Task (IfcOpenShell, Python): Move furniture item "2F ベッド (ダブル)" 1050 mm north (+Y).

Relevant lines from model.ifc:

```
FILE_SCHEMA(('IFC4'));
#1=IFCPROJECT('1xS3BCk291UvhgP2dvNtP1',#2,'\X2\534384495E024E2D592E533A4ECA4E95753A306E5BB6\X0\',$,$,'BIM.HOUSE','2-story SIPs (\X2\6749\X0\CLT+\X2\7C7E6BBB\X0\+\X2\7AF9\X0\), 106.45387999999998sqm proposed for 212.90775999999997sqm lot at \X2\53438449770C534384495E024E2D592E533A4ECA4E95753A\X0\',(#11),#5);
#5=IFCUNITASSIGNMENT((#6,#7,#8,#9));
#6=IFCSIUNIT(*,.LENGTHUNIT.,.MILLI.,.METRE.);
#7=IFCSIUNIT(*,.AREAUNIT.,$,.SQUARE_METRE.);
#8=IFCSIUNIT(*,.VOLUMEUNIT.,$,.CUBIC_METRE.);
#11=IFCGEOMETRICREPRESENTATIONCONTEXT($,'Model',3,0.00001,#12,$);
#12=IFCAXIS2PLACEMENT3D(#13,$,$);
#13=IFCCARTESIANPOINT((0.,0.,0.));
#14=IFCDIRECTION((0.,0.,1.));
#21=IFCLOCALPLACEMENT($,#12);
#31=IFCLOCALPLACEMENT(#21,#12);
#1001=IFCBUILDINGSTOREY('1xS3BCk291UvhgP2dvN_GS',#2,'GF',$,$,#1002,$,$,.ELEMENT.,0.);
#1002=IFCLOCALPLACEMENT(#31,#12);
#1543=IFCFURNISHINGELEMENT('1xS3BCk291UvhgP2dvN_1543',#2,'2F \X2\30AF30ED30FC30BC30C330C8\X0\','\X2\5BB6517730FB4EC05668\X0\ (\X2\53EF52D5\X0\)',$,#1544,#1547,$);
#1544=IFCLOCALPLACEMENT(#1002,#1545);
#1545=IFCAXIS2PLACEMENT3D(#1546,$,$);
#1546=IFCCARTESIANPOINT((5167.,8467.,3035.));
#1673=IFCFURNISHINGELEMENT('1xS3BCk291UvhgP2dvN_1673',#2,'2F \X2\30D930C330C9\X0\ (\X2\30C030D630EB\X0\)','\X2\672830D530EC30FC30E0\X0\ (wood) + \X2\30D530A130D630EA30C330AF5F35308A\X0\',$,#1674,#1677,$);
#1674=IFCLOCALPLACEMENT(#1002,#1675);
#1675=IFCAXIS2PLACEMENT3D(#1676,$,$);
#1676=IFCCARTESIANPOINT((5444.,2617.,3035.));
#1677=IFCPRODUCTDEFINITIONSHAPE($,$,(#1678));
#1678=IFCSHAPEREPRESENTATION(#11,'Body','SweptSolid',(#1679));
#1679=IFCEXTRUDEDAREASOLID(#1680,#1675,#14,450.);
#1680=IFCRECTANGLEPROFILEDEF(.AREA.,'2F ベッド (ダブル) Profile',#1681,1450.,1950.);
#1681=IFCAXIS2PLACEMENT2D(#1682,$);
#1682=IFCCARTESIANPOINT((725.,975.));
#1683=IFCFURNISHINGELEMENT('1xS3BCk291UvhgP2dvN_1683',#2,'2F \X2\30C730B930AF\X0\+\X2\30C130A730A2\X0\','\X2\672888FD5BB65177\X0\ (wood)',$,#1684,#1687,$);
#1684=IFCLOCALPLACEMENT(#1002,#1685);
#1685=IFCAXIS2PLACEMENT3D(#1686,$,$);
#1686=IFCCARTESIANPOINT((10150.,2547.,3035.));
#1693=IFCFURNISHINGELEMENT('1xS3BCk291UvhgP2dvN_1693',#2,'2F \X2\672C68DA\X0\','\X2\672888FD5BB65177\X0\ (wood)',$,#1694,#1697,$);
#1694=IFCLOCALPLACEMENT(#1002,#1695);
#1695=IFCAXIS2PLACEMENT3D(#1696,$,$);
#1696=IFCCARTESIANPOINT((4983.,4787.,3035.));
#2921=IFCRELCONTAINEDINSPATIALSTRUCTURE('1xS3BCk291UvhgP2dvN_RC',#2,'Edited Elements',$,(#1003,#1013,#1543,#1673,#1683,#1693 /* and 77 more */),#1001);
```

```python
import ifcopenshell
import ifcopenshell.api.geometry
import ifcopenshell.util.placement
import ifcopenshell.util.unit

model = ifcopenshell.open("model.ifc")
unit_scale = ifcopenshell.util.unit.calculate_unit_scale(model)

item = model.by_guid("1xS3BCk291UvhgP2dvN_1673")
matrix = ifcopenshell.util.placement.get_local_placement(item.ObjectPlacement)
matrix[1, 3] += 1.05 / unit_scale
ifcopenshell.api.geometry.edit_object_placement(model, product=item, matrix=matrix, is_si=False)

print(ifcopenshell.util.placement.get_local_placement(item.ObjectPlacement).round(3) + 0.0)

model.write("model_rev.ifc")
```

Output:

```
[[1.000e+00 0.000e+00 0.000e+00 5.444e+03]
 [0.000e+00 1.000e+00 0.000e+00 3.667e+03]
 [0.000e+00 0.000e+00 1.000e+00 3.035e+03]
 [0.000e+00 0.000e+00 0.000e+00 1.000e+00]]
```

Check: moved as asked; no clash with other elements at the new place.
